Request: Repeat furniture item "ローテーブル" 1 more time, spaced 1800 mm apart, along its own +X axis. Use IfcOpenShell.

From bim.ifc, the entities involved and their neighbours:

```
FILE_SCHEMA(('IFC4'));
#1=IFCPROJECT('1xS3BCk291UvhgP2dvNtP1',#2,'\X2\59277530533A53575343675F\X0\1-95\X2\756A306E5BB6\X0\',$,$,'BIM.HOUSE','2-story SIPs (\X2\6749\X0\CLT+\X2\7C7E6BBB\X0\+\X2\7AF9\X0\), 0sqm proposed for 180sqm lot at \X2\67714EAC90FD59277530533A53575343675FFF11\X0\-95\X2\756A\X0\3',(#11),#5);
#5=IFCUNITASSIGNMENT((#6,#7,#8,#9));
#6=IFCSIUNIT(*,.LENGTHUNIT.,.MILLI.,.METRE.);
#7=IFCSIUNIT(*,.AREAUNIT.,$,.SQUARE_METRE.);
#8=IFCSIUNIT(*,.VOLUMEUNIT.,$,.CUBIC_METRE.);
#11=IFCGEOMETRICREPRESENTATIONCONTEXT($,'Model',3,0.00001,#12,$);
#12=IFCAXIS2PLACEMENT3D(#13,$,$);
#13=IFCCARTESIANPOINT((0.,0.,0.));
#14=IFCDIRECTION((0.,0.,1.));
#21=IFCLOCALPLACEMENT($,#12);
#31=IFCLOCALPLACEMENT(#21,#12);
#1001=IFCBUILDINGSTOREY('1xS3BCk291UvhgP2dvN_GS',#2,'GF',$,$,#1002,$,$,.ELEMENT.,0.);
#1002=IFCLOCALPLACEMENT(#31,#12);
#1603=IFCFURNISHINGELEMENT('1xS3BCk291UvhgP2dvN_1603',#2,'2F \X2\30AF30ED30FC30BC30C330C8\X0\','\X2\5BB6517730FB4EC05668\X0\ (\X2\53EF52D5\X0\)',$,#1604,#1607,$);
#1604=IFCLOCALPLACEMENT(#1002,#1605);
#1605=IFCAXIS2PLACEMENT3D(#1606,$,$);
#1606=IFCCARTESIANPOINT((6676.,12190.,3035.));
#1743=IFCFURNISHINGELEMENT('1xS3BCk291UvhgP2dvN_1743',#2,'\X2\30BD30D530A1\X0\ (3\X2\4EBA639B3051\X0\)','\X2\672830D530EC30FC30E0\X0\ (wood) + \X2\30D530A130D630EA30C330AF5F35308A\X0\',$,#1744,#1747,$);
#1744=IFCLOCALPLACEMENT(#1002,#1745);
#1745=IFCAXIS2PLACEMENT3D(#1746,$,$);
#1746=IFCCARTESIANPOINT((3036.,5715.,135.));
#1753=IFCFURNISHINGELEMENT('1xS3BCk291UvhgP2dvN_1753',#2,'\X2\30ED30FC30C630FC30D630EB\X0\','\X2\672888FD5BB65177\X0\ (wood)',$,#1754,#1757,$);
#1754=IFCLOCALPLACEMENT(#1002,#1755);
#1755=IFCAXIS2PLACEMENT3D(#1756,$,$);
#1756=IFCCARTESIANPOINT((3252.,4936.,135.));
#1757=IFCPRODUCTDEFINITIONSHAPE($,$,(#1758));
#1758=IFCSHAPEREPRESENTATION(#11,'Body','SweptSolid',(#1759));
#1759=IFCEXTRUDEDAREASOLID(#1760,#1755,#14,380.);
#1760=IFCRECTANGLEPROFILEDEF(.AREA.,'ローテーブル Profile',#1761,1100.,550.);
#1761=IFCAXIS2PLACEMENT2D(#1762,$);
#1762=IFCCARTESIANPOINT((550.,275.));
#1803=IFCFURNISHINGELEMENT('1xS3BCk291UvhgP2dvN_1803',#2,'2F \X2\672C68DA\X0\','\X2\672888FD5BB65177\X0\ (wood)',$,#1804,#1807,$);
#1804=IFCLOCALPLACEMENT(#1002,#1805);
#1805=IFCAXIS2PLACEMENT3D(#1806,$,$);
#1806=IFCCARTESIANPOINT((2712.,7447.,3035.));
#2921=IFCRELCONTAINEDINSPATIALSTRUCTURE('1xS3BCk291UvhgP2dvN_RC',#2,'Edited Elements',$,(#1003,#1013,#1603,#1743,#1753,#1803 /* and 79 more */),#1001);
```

```python
import ifcopenshell
import ifcopenshell.api.geometry
import ifcopenshell.api.root
import ifcopenshell.util.element
import ifcopenshell.util.placement

model = ifcopenshell.open("bim.ifc")


def reuse_history(source, copy):
    """copy_class also copies each property set's owner history, people and application; keep the originals."""
    for rel in copy.IsDefinedBy:
        if rel.is_a("IfcRelDefinesByProperties") and (history := rel.RelatingPropertyDefinition.OwnerHistory):
            rel.RelatingPropertyDefinition.OwnerHistory = source.OwnerHistory
            ifcopenshell.util.element.remove_deep2(model, history)


source = model.by_guid("1xS3BCk291UvhgP2dvN_1753")
base = ifcopenshell.util.placement.get_local_placement(source.ObjectPlacement)
step = base[:3, 0] * 1800.0

for i in range(1, 2):
    copy = ifcopenshell.api.root.copy_class(model, product=source)
    copy.Representation = ifcopenshell.util.element.copy_deep(
        model, source.Representation, exclude=["IfcGeometricRepresentationContext", "IfcRepresentationMap"]
    )
    reuse_history(source, copy)
    matrix = base.copy()
    matrix[:3, 3] += i * step
    print("added at", matrix[:3, 3].round(3) + 0.0)
    ifcopenshell.api.geometry.edit_object_placement(model, product=copy, matrix=matrix, is_si=False)

model.write("bim_updated.ifc")
```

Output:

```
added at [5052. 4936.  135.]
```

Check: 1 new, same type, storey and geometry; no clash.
